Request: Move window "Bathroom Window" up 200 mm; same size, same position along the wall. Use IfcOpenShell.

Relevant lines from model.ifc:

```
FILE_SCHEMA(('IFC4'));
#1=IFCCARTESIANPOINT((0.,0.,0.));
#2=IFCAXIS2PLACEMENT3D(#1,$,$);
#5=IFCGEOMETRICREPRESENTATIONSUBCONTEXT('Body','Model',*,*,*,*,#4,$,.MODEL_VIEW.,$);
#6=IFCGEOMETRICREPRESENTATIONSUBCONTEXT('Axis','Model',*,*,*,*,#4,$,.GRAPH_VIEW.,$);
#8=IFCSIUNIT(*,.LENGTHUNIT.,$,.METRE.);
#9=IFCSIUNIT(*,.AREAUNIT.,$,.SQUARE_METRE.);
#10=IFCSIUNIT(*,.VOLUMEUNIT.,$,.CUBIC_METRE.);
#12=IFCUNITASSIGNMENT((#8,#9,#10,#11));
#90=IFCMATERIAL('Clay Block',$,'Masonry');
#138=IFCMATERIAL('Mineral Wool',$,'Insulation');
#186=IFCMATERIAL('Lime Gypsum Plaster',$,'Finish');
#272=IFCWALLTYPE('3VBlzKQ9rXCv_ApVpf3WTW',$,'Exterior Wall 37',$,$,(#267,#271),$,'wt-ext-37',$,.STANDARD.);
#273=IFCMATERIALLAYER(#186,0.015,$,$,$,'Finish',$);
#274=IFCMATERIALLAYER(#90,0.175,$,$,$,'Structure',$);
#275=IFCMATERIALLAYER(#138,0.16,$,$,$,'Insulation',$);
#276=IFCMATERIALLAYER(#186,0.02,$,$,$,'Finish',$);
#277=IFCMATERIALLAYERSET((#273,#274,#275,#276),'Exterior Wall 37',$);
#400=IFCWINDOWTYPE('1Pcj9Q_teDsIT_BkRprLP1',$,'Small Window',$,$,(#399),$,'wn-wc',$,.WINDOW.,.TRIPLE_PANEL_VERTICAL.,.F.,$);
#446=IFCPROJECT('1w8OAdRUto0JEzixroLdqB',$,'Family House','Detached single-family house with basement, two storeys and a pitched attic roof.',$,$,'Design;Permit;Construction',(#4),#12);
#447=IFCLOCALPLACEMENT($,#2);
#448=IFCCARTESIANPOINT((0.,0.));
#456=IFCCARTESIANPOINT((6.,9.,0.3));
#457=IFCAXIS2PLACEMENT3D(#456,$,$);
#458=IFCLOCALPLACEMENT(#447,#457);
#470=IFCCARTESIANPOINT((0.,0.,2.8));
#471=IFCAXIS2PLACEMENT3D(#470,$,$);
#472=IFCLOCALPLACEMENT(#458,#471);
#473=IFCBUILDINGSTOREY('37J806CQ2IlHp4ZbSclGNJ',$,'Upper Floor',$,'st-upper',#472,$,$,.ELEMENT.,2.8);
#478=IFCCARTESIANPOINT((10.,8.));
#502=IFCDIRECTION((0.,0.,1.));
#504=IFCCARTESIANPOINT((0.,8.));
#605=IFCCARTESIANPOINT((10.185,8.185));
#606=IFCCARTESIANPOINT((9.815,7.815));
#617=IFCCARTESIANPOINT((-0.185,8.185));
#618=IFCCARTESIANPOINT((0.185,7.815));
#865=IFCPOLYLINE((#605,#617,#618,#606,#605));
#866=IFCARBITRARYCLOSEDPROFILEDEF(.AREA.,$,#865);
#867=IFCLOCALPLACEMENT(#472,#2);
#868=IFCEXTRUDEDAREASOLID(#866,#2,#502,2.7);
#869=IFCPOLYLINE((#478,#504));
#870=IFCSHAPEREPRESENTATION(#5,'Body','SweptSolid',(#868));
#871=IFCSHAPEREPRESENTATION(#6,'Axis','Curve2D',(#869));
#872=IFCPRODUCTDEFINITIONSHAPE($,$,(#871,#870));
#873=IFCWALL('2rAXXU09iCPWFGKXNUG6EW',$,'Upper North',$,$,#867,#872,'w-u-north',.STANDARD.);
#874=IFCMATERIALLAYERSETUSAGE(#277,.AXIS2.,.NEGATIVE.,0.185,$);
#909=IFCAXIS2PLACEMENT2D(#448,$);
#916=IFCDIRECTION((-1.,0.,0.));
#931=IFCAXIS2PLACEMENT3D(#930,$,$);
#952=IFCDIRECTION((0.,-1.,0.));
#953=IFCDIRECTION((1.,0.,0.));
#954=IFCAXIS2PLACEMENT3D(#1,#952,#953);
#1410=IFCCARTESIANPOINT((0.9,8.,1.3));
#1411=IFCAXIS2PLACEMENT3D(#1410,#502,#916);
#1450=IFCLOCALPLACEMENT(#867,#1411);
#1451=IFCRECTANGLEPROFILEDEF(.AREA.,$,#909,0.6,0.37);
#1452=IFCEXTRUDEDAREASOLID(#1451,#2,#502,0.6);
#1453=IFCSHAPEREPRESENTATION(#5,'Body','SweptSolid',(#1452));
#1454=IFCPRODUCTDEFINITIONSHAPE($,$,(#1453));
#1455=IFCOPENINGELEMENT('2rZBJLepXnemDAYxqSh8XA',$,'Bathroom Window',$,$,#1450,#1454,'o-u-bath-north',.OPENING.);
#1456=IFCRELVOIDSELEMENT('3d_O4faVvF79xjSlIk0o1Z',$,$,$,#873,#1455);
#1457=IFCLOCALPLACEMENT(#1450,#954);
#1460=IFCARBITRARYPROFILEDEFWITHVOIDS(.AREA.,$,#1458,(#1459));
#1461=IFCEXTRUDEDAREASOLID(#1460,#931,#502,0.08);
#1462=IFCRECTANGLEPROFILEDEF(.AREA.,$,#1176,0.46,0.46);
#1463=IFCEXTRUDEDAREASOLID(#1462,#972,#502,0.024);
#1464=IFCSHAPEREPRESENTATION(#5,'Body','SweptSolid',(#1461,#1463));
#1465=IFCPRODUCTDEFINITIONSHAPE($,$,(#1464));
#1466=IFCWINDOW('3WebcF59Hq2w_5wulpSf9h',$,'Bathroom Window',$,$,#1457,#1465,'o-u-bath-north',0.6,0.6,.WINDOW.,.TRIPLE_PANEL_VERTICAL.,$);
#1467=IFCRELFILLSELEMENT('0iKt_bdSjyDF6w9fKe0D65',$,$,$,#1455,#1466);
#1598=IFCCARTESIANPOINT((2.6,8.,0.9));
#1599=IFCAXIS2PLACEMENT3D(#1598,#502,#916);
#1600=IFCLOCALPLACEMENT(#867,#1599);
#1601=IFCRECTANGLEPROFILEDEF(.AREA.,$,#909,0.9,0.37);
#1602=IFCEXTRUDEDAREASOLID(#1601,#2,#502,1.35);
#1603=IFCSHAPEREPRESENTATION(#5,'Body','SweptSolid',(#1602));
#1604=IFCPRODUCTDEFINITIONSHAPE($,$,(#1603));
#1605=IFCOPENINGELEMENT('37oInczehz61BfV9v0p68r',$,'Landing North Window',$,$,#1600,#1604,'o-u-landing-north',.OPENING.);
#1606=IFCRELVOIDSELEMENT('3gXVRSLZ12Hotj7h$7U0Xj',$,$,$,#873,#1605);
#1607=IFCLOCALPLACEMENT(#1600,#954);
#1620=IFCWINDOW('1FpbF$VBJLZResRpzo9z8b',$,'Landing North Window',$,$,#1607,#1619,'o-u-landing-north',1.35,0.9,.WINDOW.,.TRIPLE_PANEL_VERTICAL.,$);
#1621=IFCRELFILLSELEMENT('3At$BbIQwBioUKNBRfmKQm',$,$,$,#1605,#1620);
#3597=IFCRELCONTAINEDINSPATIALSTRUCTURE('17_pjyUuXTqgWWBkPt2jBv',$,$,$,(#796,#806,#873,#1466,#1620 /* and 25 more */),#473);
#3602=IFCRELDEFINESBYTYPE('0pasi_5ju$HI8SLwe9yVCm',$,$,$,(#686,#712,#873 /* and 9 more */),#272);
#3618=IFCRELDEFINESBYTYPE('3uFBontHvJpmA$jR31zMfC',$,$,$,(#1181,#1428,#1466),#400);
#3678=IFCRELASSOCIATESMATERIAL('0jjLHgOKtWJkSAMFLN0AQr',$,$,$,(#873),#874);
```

```python
import numpy as np
import ifcopenshell
import ifcopenshell.api.geometry
import ifcopenshell.util.placement
import ifcopenshell.util.unit

model = ifcopenshell.open("model.ifc")
unit_scale = ifcopenshell.util.unit.calculate_unit_scale(model)

window = model.by_guid("3WebcF59Hq2w_5wulpSf9h")
opening = window.FillsVoids[0].RelatingOpeningElement
dz = 0.2

shift = np.array([0.0, 0.0, dz])
# The window is placed relative to its opening, so it follows when the opening moves.
matrix = ifcopenshell.util.placement.get_local_placement(opening.ObjectPlacement)
matrix[:3, 3] += shift
ifcopenshell.api.geometry.edit_object_placement(
    model, product=opening, matrix=matrix, is_si=False, should_transform_children=True
)

print(f"moved by {dz * unit_scale:+.3f} m")

model.write("model_updated.ifc")
```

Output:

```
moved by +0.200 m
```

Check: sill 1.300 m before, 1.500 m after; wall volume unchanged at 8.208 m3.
